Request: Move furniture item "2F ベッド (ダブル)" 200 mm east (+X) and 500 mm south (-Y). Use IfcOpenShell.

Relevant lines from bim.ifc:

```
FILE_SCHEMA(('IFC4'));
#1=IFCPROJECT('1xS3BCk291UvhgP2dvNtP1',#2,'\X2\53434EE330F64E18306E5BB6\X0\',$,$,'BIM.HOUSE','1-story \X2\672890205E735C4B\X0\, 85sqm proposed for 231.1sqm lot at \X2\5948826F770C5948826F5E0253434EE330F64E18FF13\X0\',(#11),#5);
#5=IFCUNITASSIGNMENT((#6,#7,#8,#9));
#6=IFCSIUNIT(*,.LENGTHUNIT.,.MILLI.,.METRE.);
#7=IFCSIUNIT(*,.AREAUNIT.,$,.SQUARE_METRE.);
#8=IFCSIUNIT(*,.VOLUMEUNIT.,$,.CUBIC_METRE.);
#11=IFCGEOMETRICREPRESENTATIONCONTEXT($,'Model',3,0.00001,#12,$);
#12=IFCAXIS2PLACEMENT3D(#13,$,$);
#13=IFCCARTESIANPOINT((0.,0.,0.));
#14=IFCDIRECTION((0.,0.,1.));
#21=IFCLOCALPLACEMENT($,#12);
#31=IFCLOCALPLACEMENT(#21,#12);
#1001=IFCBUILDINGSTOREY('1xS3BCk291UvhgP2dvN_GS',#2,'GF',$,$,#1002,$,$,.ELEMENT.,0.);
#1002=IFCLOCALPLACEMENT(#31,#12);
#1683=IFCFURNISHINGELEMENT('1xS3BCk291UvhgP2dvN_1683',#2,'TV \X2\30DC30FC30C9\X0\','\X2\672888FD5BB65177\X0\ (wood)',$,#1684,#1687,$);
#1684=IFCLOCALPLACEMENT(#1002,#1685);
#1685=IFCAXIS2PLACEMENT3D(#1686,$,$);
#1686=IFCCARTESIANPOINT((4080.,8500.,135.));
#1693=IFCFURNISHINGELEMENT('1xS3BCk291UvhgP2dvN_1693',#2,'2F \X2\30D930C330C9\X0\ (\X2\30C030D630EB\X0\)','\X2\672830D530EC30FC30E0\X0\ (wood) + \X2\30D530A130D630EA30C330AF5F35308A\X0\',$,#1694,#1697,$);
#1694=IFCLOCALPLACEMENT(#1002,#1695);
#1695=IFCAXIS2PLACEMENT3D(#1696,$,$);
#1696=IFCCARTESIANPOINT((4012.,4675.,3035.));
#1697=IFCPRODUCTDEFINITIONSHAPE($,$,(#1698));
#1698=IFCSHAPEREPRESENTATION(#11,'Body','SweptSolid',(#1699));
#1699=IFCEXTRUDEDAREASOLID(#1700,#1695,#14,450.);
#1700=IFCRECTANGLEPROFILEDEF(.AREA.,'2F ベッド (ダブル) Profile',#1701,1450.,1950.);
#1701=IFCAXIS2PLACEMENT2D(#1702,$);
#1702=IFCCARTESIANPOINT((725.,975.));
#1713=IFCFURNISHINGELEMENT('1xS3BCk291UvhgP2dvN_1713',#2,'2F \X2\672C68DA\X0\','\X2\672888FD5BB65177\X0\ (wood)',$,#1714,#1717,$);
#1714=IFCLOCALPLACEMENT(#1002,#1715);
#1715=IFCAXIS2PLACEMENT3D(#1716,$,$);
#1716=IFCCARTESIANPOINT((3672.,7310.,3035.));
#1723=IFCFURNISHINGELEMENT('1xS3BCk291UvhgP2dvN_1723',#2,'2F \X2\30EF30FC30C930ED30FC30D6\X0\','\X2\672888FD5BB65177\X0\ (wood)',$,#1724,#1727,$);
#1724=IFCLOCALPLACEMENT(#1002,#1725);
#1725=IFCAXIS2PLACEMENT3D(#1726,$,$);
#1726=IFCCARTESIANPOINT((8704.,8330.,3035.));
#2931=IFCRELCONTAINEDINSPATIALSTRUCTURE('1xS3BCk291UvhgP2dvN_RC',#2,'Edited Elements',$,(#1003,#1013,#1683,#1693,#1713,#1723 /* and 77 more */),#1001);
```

```python
import ifcopenshell
import ifcopenshell.api.geometry
import ifcopenshell.util.placement

model = ifcopenshell.open("bim.ifc")

item = model.by_guid("1xS3BCk291UvhgP2dvN_1693")
matrix = ifcopenshell.util.placement.get_local_placement(item.ObjectPlacement)
matrix[0, 3] += 200.0
matrix[1, 3] -= 500.0
ifcopenshell.api.geometry.edit_object_placement(model, product=item, matrix=matrix, is_si=False)

print(ifcopenshell.util.placement.get_local_placement(item.ObjectPlacement).round(3) + 0.0)

model.write("bim_updated.ifc")
```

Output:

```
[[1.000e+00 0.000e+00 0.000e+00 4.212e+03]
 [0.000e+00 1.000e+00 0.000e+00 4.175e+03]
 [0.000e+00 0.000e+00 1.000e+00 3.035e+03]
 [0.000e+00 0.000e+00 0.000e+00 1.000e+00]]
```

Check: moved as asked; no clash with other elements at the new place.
